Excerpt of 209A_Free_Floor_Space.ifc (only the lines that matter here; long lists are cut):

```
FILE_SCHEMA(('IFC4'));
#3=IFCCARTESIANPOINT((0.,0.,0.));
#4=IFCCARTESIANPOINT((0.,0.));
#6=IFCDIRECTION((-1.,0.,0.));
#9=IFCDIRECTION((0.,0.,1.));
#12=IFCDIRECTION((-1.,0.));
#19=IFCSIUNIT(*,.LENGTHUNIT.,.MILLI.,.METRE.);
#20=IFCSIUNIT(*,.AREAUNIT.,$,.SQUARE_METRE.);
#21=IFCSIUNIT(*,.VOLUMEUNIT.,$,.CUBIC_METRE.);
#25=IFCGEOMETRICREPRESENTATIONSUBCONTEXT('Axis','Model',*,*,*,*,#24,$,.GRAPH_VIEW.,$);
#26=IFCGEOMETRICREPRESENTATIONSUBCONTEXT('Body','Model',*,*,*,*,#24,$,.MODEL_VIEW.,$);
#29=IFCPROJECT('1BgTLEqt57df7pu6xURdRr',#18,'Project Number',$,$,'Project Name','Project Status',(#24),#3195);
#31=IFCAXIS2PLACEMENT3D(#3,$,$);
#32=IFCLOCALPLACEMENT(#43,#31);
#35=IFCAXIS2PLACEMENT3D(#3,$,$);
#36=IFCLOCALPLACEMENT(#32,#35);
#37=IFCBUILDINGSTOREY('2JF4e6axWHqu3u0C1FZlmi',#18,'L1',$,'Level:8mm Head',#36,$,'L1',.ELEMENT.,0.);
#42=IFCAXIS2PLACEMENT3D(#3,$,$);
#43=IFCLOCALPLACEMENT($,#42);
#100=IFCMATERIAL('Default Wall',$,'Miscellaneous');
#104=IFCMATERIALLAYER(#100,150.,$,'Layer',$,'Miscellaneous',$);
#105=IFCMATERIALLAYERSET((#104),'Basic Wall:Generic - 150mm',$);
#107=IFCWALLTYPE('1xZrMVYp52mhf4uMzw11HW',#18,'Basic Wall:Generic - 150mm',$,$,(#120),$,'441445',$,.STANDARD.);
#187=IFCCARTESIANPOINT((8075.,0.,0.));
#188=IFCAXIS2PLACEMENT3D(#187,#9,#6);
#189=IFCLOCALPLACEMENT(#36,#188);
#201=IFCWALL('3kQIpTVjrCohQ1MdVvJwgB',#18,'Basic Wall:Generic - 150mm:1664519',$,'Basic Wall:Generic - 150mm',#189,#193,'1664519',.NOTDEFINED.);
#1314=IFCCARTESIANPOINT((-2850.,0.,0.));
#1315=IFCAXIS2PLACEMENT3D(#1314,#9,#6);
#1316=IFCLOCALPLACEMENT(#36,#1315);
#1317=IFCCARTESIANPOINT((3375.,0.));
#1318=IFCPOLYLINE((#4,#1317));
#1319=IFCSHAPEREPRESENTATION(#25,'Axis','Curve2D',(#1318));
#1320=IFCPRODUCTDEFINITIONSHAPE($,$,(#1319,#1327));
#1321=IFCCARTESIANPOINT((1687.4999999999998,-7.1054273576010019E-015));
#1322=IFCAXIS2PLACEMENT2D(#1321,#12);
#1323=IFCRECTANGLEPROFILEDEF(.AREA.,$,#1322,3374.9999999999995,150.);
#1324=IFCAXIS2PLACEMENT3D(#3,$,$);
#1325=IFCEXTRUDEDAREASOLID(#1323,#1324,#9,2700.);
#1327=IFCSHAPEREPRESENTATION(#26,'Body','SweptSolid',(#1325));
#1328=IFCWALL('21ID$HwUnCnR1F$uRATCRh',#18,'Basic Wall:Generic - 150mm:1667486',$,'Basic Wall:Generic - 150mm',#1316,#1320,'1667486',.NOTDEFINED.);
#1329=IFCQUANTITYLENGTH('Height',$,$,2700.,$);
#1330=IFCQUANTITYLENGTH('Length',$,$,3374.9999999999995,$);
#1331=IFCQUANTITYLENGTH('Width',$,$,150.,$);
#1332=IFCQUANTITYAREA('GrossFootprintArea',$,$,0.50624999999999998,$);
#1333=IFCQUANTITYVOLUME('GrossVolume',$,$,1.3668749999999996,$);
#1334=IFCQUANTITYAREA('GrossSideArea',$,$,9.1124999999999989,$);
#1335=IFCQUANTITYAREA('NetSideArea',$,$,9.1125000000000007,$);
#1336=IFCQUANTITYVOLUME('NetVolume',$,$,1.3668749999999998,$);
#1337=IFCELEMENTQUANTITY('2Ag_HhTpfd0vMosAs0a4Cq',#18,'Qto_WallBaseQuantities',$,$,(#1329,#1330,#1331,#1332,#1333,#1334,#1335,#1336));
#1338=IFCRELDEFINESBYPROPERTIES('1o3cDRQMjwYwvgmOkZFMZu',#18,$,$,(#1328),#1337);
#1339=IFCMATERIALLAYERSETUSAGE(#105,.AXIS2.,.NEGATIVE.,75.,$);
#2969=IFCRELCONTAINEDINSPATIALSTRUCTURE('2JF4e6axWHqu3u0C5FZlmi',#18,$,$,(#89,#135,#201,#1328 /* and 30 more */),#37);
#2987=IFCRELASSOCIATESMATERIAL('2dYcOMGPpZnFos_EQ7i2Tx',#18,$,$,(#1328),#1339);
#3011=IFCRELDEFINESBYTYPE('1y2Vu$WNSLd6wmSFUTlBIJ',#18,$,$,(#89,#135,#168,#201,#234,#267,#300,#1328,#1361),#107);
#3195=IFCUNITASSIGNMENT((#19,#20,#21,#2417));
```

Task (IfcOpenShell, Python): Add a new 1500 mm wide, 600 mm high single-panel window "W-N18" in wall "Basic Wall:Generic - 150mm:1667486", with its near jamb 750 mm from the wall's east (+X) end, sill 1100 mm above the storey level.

```python
import numpy as np
import ifcopenshell
import ifcopenshell.api.feature
import ifcopenshell.api.geometry
import ifcopenshell.api.pset
import ifcopenshell.api.root
import ifcopenshell.api.spatial
import ifcopenshell.geom
import ifcopenshell.util.element
import ifcopenshell.util.placement
import ifcopenshell.util.representation
import ifcopenshell.util.shape
import ifcopenshell.util.unit

model = ifcopenshell.open("209A_Free_Floor_Space.ifc")
unit_scale = ifcopenshell.util.unit.calculate_unit_scale(model)
area_scale = ifcopenshell.util.unit.calculate_unit_scale(model, "AREAUNIT")
volume_scale = ifcopenshell.util.unit.calculate_unit_scale(model, "VOLUMEUNIT")
settings = ifcopenshell.geom.settings()


def volume(element):
    """Net volume in cubic metres, openings subtracted."""
    shape = ifcopenshell.geom.create_shape(settings, element)
    return ifcopenshell.util.shape.get_volume(shape.geometry)


wall = model.by_guid("21ID$HwUnCnR1F$uRATCRh")
storey = ifcopenshell.util.element.get_container(wall, ifc_class="IfcBuildingStorey")
context = ifcopenshell.util.representation.get_context(model, "Model", "Body", "MODEL_VIEW")
before = volume(wall)

width, height, from_end, sill = 1.5, 0.6, 0.75, 1.1  # metres

# The wall runs along its own X axis, and the end named is its -X end.
wall_shape = ifcopenshell.geom.create_shape(settings, wall)
x, y, z = ifcopenshell.util.shape.get_vertices(wall_shape.geometry).T
start = x.min() + from_end
face, thickness = float(y.min()), float(y.max() - y.min())
wall_matrix = ifcopenshell.util.placement.get_local_placement(wall.ObjectPlacement)
level = ifcopenshell.util.placement.get_local_placement(storey.ObjectPlacement)[2, 3]


def in_wall(x, y):
    """Placement at x, y metres in the wall's axes, at sill height."""
    matrix = wall_matrix.copy()
    matrix[:, 3] = wall_matrix @ np.array([x / unit_scale, y / unit_scale, 0.0, 1.0])
    matrix[2, 3] = level + sill / unit_scale
    return matrix


# Opening: a box that overshoots both wall faces by 50 mm.
opening = ifcopenshell.api.root.create_entity(model, ifc_class="IfcOpeningElement", predefined_type="OPENING")
box = ifcopenshell.api.geometry.add_wall_representation(
    model, context=context, length=width, height=height, thickness=thickness + 0.1
)
ifcopenshell.api.geometry.assign_representation(model, product=opening, representation=box)
ifcopenshell.api.geometry.edit_object_placement(model, product=opening, matrix=in_wall(start, face - 0.05), is_si=False)
ifcopenshell.api.feature.add_feature(model, feature=opening, element=wall)

window = ifcopenshell.api.root.create_entity(model, ifc_class="IfcWindow", name="W-N18", predefined_type="WINDOW")
window.OverallWidth, window.OverallHeight = width / unit_scale, height / unit_scale
window.PartitioningType = "SINGLE_PANEL"
body = ifcopenshell.api.geometry.add_window_representation(
    model,
    context=context,
    overall_width=window.OverallWidth,
    overall_height=window.OverallHeight,
    partition_type="SINGLE_PANEL",
)
ifcopenshell.api.geometry.assign_representation(model, product=window, representation=body)
ifcopenshell.api.spatial.assign_container(model, products=[window], relating_structure=storey)
ifcopenshell.api.feature.add_filling(model, opening=opening, element=window)

# Centre the window in the wall's thickness.
ifcopenshell.api.geometry.edit_object_placement(model, product=window, matrix=in_wall(start, face), is_si=False)
window_shape = ifcopenshell.geom.create_shape(settings, window)
depth = ifcopenshell.util.shape.get_vertices(window_shape.geometry)[:, 1]
offset = face + thickness / 2 - (depth.min() + depth.max()) / 2
ifcopenshell.api.geometry.edit_object_placement(model, product=window, matrix=in_wall(start, offset), is_si=False)

after = volume(wall)

# Update the wall's stored quantities.
qto = model.by_id(ifcopenshell.util.element.get_pset(wall, "Qto_WallBaseQuantities", should_inherit=False)["id"])
ifcopenshell.api.pset.edit_qto(model, qto=qto, properties={
    "NetSideArea": after / thickness / area_scale,
    "NetVolume": after / volume_scale,
})

print(f"wall volume {before:.3f} -> {after:.3f} m3")

model.write("209A_Free_Floor_Space-out.ifc")
```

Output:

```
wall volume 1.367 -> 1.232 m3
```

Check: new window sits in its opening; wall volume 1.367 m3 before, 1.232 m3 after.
